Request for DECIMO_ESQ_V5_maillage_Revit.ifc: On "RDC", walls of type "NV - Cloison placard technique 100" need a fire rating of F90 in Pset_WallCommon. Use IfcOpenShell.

First a look at what the model holds.

```python
import ifcopenshell
import ifcopenshell.util.element

model = ifcopenshell.open("DECIMO_ESQ_V5_maillage_Revit.ifc")
print(model.schema)
storey = next(s for s in model.by_type("IfcBuildingStorey") if s.Name == "RDC")
walls = [e for e in ifcopenshell.util.element.get_decomposition(storey) if e.is_a("IfcWall")]
seen = {}
for e in walls:
    element_type = ifcopenshell.util.element.get_type(e)
    key = (element_type.Name if element_type != e and element_type else None, ifcopenshell.util.element.get_pset(e, "Pset_WallCommon", "FireRating"))
    seen[key] = seen.get(key, 0) + 1
for (name, value), count in sorted(seen.items(), key=str):
    print(count, "x", name, "|", value)
```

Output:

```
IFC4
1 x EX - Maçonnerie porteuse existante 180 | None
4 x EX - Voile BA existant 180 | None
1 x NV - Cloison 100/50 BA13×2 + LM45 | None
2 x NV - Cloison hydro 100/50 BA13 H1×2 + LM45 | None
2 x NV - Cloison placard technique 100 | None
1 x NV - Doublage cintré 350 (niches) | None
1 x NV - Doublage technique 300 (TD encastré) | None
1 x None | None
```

```python
import ifcopenshell
import ifcopenshell.api.pset
import ifcopenshell.util.element

model = ifcopenshell.open("DECIMO_ESQ_V5_maillage_Revit.ifc")

storey = next(s for s in model.by_type("IfcBuildingStorey") if s.Name == "RDC")
walls = [e for e in ifcopenshell.util.element.get_decomposition(storey) if e.is_a("IfcWall")]

count = 0
for e in walls:
    element_type = ifcopenshell.util.element.get_type(e)
    if element_type in (None, e) or element_type.Name != "NV - Cloison placard technique 100":
        continue
    # add_pset returns the element's existing set when there is one.
    pset = ifcopenshell.api.pset.add_pset(model, product=e, name="Pset_WallCommon")
    ifcopenshell.api.pset.edit_pset(model, pset=pset, properties={"FireRating": "F90"})
    count += 1

print(count, "walls updated")

model.write("DECIMO_ESQ_V5_maillage_Revit_edited.ifc")
```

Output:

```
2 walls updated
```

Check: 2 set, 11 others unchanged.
